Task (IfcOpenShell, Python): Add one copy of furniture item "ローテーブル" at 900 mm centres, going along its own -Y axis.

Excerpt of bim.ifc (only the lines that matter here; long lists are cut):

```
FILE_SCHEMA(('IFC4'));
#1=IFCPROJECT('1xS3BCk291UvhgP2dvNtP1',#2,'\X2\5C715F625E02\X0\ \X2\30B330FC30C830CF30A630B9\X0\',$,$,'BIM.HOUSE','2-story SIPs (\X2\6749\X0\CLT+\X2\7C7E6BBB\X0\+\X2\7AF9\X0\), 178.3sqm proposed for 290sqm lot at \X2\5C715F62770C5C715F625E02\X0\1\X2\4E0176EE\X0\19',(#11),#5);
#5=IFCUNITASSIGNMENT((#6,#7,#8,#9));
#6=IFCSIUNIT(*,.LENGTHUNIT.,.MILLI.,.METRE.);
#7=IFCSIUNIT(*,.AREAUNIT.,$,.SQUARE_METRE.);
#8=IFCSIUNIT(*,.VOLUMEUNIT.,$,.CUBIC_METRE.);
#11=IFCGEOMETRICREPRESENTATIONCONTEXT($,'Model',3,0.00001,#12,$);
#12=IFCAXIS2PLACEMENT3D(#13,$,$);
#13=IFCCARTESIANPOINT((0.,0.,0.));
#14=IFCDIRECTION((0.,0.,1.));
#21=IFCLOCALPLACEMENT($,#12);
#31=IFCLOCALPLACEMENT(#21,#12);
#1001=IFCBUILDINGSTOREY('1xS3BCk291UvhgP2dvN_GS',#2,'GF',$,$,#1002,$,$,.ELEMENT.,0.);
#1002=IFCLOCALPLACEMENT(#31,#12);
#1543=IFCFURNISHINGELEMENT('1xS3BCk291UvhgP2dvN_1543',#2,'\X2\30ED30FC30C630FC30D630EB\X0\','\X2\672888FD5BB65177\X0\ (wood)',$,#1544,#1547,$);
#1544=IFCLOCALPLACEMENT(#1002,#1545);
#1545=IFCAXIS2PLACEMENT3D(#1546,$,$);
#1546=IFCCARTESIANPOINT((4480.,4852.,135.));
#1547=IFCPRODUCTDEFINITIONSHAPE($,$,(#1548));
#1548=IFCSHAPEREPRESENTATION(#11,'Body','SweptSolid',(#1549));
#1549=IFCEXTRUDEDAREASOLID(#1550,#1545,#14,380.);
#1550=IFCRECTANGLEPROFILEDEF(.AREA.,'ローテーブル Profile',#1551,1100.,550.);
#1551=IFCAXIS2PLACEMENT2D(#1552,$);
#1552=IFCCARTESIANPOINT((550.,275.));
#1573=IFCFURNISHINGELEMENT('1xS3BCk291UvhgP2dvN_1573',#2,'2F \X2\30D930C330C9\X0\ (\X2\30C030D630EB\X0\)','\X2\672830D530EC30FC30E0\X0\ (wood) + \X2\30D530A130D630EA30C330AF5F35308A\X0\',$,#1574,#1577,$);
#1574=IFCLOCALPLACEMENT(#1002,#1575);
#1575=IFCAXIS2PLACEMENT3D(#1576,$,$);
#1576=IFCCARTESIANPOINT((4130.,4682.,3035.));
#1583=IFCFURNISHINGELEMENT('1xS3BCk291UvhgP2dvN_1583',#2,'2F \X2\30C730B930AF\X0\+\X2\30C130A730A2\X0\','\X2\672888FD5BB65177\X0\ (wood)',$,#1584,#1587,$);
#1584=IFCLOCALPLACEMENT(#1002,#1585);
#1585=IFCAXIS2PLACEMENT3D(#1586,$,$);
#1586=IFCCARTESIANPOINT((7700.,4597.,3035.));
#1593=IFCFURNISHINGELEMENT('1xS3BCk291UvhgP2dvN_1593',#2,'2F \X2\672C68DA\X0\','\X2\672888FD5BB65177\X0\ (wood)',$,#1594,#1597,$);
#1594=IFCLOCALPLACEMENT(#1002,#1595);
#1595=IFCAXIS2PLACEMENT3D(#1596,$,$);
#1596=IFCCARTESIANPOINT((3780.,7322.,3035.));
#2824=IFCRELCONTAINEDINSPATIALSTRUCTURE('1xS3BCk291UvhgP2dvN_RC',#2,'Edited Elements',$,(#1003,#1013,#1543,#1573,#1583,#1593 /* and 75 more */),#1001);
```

```python
import ifcopenshell
import ifcopenshell.api.geometry
import ifcopenshell.api.root
import ifcopenshell.util.element
import ifcopenshell.util.placement
import ifcopenshell.util.unit

model = ifcopenshell.open("bim.ifc")
unit_scale = ifcopenshell.util.unit.calculate_unit_scale(model)


def reuse_history(source, copy):
    """copy_class also copies each property set's owner history, people and application; keep the originals."""
    for rel in copy.IsDefinedBy:
        if rel.is_a("IfcRelDefinesByProperties") and (history := rel.RelatingPropertyDefinition.OwnerHistory):
            rel.RelatingPropertyDefinition.OwnerHistory = source.OwnerHistory
            ifcopenshell.util.element.remove_deep2(model, history)


source = model.by_guid("1xS3BCk291UvhgP2dvN_1543")
base = ifcopenshell.util.placement.get_local_placement(source.ObjectPlacement)
step = -base[:3, 1] * 0.9 / unit_scale

for i in range(1, 2):
    copy = ifcopenshell.api.root.copy_class(model, product=source)
    copy.Representation = ifcopenshell.util.element.copy_deep(
        model, source.Representation, exclude=["IfcGeometricRepresentationContext", "IfcRepresentationMap"]
    )
    reuse_history(source, copy)
    matrix = base.copy()
    matrix[:3, 3] += i * step
    print("added at", matrix[:3, 3].round(3) + 0.0)
    ifcopenshell.api.geometry.edit_object_placement(model, product=copy, matrix=matrix, is_si=False)

model.write("bim-out.ifc")
```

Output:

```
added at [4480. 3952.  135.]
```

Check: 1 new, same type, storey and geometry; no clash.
